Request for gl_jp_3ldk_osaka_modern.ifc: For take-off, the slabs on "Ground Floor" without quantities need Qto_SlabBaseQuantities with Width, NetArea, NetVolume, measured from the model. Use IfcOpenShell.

First a look at what the model holds.

```python
import ifcopenshell
import ifcopenshell.util.element
import ifcopenshell.util.unit

model = ifcopenshell.open("gl_jp_3ldk_osaka_modern.ifc")
print(model.schema)
for unit_type in ("LENGTHUNIT", "AREAUNIT", "VOLUMEUNIT"):
    print(unit_type, ifcopenshell.util.unit.calculate_unit_scale(model, unit_type))
storey = next(s for s in model.by_type("IfcBuildingStorey") if s.Name == "Ground Floor")
slabs = [e for e in ifcopenshell.util.element.get_decomposition(storey) if e.is_a("IfcSlab")]
for e in sorted(slabs, key=lambda e: e.id()):
    print(e.id(), e.is_a(), e.Name, list(ifcopenshell.util.element.get_psets(e, qtos_only=True)), sep=" | ")
```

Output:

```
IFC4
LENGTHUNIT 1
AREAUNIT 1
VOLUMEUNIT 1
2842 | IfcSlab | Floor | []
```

```python
import ifcopenshell
import ifcopenshell.api.pset
import ifcopenshell.geom
import ifcopenshell.util.element
import ifcopenshell.util.shape
import ifcopenshell.util.unit

model = ifcopenshell.open("gl_jp_3ldk_osaka_modern.ifc")
unit_scale = ifcopenshell.util.unit.calculate_unit_scale(model)
area_scale = ifcopenshell.util.unit.calculate_unit_scale(model, "AREAUNIT")
volume_scale = ifcopenshell.util.unit.calculate_unit_scale(model, "VOLUMEUNIT")
settings = ifcopenshell.geom.settings()

storey = next(s for s in model.by_type("IfcBuildingStorey") if s.Name == "Ground Floor")
slabs = [e for e in ifcopenshell.util.element.get_decomposition(storey) if e.is_a("IfcSlab")]

for e in sorted(slabs, key=lambda e: e.id()):
    if ifcopenshell.util.element.get_psets(e, qtos_only=True, should_inherit=False):
        continue
    # Geometry comes back in metres, in the element's own axes.
    shape = ifcopenshell.geom.create_shape(settings, e)
    values = {
        "Width": ifcopenshell.util.shape.get_z(shape.geometry) / unit_scale,
        "NetArea": ifcopenshell.util.shape.get_footprint_area(shape.geometry) / area_scale,
        "NetVolume": ifcopenshell.util.shape.get_volume(shape.geometry) / volume_scale,
    }
    qto = ifcopenshell.api.pset.add_qto(model, product=e, name="Qto_SlabBaseQuantities")
    ifcopenshell.api.pset.edit_qto(model, qto=qto, properties=values)
    print(e.id(), {k: round(v, 3) for k, v in values.items()})

model.write("gl_jp_3ldk_osaka_modern_edited.ifc")
```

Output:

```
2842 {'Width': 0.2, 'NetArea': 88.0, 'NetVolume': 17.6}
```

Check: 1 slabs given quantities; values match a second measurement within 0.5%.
